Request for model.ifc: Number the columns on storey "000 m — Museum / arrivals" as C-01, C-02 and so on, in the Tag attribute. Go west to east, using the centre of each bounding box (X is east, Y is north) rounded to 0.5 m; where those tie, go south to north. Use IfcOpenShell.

First a look at what the model holds.

```python
import ifcopenshell
import ifcopenshell.util.element
import ifcopenshell.util.placement

model = ifcopenshell.open("model.ifc")
print(model.schema)
storey = next(s for s in model.by_type("IfcBuildingStorey") if s.Name == "000 m — Museum / arrivals")
columns = [e for e in ifcopenshell.util.element.get_decomposition(storey) if e.is_a("IfcColumn")]
for e in sorted(columns, key=lambda e: e.id()):
    origin = ifcopenshell.util.placement.get_local_placement(e.ObjectPlacement)[:3, 3]
    print(e.id(), e.Tag, e.Name, origin.round(2) + 0.0, sep=" | ")
```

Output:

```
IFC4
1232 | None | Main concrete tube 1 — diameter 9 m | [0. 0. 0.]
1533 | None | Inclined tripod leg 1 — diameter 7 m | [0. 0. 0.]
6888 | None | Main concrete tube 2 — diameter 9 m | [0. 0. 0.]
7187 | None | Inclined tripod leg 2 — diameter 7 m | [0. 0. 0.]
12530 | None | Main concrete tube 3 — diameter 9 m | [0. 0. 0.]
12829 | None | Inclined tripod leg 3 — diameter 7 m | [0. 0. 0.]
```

```python
import ifcopenshell
import ifcopenshell.geom
import ifcopenshell.util.element
import ifcopenshell.util.shape

model = ifcopenshell.open("model.ifc")
settings = ifcopenshell.geom.settings()
settings.set("use-world-coords", True)


def centre(element):
    shape = ifcopenshell.geom.create_shape(settings, element)
    return ifcopenshell.util.shape.get_bbox_centroid(shape.geometry)


storey = next(s for s in model.by_type("IfcBuildingStorey") if s.Name == "000 m — Museum / arrivals")
columns = [e for e in ifcopenshell.util.element.get_decomposition(storey) if e.is_a("IfcColumn")]

# Insertion points can sit at a corner or the storey origin, so sort by the geometry (in metres).
centres = {e: centre(e) for e in columns}
columns.sort(key=lambda e: (round(centres[e][0] / 0.5), centres[e][1]))

for i, e in enumerate(columns, start=1):
    number = f"C-{i:02d}"
    e.Tag = number
    print(e.id(), number)

model.write("model-out.ifc")
```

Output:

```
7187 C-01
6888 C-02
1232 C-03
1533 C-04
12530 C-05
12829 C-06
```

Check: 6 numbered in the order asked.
